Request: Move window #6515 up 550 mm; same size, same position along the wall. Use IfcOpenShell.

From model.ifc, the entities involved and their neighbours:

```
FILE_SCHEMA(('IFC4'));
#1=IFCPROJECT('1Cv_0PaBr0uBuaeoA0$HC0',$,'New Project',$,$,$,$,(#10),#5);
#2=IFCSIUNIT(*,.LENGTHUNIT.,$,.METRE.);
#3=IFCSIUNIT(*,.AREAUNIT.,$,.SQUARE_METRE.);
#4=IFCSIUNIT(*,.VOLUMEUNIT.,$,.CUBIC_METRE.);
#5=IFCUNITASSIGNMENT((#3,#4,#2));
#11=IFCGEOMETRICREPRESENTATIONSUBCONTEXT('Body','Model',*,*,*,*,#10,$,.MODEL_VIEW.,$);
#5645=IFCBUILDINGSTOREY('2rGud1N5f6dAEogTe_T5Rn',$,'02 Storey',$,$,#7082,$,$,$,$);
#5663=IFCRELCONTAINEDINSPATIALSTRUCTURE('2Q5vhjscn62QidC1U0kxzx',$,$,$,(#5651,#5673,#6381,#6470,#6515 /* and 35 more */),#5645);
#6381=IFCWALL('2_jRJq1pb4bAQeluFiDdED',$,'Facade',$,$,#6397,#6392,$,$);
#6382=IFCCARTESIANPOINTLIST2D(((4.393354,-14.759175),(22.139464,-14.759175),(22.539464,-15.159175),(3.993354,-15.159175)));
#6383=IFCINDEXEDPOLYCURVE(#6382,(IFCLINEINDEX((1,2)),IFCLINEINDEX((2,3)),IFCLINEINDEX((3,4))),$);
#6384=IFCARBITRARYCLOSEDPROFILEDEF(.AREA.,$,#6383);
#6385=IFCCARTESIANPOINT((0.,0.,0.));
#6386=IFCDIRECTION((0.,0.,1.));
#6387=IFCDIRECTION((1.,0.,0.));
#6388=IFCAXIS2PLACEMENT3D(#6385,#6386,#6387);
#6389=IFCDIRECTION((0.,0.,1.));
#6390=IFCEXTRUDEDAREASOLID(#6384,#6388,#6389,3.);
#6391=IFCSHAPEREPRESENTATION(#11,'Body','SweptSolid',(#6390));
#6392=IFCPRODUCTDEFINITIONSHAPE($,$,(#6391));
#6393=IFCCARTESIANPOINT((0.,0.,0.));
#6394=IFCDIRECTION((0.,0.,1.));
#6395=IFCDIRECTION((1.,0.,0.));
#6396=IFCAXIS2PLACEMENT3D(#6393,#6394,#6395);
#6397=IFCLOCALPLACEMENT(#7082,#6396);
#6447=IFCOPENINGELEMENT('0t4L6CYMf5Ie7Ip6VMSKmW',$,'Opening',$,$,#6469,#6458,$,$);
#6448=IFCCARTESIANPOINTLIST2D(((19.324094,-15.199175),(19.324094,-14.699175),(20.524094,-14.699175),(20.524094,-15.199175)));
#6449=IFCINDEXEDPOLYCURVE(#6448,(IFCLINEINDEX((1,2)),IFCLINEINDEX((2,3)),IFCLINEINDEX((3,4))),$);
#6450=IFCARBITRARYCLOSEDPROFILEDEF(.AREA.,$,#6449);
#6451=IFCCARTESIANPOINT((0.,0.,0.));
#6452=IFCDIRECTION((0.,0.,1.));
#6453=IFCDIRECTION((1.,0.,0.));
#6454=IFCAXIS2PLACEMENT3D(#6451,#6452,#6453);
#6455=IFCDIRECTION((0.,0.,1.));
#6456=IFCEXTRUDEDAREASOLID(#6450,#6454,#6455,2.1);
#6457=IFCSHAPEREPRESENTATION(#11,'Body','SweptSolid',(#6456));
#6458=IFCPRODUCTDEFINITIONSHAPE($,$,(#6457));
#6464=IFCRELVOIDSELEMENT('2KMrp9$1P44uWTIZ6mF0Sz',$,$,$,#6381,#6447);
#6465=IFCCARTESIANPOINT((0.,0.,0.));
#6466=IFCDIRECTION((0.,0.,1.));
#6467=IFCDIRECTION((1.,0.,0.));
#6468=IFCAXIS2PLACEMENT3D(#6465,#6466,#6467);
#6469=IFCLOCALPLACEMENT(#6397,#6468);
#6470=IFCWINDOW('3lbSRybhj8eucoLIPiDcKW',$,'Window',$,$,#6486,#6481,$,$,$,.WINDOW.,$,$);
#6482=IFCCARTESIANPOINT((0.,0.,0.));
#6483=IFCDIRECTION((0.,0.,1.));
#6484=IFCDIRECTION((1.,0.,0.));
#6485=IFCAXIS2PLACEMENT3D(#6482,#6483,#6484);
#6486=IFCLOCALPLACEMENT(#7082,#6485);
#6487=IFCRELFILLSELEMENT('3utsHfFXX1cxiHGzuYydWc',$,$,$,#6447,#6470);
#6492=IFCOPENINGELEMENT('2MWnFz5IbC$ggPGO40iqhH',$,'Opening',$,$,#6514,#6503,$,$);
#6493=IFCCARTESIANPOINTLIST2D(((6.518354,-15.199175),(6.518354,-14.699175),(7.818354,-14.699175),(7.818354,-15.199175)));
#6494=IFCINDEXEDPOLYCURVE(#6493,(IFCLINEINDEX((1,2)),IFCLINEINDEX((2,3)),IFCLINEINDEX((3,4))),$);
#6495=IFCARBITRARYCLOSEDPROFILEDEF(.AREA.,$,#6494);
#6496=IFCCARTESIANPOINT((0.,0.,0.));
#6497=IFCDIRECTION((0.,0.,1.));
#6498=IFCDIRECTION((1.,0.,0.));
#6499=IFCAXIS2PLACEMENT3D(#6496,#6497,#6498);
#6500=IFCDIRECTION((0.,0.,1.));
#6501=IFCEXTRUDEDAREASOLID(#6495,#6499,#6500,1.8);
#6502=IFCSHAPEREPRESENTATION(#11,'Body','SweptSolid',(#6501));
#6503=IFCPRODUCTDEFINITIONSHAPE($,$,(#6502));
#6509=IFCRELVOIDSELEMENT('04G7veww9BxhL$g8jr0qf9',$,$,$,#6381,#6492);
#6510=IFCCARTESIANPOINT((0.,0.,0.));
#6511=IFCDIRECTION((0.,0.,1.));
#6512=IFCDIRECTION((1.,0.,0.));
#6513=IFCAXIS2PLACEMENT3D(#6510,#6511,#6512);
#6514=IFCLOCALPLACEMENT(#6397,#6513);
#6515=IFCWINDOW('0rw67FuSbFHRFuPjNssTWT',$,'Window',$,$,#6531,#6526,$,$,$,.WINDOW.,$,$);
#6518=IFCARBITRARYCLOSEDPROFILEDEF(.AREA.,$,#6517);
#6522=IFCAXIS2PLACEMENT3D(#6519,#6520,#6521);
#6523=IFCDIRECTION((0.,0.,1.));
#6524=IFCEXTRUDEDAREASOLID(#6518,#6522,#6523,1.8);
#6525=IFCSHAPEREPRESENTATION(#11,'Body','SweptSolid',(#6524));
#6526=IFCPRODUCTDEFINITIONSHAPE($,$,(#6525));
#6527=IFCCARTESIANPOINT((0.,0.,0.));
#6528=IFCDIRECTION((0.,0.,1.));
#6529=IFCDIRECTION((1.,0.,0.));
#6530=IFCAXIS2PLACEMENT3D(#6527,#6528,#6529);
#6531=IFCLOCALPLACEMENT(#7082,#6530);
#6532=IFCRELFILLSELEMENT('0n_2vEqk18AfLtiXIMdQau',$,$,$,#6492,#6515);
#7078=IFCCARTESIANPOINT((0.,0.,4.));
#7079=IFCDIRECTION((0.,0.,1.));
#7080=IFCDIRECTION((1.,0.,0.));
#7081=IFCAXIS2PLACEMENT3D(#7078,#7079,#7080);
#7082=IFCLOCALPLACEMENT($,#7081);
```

```python
import numpy as np
import ifcopenshell
import ifcopenshell.api.geometry
import ifcopenshell.util.placement
import ifcopenshell.util.unit

model = ifcopenshell.open("model.ifc")
unit_scale = ifcopenshell.util.unit.calculate_unit_scale(model)

window = model.by_guid("0rw67FuSbFHRFuPjNssTWT")
opening = window.FillsVoids[0].RelatingOpeningElement
dz = 0.55 / unit_scale

shift = np.array([0.0, 0.0, dz])
# The window is not placed relative to its opening, so move both.
for product in (opening, window):
    matrix = ifcopenshell.util.placement.get_local_placement(product.ObjectPlacement)
    matrix[:3, 3] += shift
    ifcopenshell.api.geometry.edit_object_placement(model, product=product, matrix=matrix, is_si=False)

print(f"moved by {dz * unit_scale:+.3f} m")

model.write("model_edited.ifc")
```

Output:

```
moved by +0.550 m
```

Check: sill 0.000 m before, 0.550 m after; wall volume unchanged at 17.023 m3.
